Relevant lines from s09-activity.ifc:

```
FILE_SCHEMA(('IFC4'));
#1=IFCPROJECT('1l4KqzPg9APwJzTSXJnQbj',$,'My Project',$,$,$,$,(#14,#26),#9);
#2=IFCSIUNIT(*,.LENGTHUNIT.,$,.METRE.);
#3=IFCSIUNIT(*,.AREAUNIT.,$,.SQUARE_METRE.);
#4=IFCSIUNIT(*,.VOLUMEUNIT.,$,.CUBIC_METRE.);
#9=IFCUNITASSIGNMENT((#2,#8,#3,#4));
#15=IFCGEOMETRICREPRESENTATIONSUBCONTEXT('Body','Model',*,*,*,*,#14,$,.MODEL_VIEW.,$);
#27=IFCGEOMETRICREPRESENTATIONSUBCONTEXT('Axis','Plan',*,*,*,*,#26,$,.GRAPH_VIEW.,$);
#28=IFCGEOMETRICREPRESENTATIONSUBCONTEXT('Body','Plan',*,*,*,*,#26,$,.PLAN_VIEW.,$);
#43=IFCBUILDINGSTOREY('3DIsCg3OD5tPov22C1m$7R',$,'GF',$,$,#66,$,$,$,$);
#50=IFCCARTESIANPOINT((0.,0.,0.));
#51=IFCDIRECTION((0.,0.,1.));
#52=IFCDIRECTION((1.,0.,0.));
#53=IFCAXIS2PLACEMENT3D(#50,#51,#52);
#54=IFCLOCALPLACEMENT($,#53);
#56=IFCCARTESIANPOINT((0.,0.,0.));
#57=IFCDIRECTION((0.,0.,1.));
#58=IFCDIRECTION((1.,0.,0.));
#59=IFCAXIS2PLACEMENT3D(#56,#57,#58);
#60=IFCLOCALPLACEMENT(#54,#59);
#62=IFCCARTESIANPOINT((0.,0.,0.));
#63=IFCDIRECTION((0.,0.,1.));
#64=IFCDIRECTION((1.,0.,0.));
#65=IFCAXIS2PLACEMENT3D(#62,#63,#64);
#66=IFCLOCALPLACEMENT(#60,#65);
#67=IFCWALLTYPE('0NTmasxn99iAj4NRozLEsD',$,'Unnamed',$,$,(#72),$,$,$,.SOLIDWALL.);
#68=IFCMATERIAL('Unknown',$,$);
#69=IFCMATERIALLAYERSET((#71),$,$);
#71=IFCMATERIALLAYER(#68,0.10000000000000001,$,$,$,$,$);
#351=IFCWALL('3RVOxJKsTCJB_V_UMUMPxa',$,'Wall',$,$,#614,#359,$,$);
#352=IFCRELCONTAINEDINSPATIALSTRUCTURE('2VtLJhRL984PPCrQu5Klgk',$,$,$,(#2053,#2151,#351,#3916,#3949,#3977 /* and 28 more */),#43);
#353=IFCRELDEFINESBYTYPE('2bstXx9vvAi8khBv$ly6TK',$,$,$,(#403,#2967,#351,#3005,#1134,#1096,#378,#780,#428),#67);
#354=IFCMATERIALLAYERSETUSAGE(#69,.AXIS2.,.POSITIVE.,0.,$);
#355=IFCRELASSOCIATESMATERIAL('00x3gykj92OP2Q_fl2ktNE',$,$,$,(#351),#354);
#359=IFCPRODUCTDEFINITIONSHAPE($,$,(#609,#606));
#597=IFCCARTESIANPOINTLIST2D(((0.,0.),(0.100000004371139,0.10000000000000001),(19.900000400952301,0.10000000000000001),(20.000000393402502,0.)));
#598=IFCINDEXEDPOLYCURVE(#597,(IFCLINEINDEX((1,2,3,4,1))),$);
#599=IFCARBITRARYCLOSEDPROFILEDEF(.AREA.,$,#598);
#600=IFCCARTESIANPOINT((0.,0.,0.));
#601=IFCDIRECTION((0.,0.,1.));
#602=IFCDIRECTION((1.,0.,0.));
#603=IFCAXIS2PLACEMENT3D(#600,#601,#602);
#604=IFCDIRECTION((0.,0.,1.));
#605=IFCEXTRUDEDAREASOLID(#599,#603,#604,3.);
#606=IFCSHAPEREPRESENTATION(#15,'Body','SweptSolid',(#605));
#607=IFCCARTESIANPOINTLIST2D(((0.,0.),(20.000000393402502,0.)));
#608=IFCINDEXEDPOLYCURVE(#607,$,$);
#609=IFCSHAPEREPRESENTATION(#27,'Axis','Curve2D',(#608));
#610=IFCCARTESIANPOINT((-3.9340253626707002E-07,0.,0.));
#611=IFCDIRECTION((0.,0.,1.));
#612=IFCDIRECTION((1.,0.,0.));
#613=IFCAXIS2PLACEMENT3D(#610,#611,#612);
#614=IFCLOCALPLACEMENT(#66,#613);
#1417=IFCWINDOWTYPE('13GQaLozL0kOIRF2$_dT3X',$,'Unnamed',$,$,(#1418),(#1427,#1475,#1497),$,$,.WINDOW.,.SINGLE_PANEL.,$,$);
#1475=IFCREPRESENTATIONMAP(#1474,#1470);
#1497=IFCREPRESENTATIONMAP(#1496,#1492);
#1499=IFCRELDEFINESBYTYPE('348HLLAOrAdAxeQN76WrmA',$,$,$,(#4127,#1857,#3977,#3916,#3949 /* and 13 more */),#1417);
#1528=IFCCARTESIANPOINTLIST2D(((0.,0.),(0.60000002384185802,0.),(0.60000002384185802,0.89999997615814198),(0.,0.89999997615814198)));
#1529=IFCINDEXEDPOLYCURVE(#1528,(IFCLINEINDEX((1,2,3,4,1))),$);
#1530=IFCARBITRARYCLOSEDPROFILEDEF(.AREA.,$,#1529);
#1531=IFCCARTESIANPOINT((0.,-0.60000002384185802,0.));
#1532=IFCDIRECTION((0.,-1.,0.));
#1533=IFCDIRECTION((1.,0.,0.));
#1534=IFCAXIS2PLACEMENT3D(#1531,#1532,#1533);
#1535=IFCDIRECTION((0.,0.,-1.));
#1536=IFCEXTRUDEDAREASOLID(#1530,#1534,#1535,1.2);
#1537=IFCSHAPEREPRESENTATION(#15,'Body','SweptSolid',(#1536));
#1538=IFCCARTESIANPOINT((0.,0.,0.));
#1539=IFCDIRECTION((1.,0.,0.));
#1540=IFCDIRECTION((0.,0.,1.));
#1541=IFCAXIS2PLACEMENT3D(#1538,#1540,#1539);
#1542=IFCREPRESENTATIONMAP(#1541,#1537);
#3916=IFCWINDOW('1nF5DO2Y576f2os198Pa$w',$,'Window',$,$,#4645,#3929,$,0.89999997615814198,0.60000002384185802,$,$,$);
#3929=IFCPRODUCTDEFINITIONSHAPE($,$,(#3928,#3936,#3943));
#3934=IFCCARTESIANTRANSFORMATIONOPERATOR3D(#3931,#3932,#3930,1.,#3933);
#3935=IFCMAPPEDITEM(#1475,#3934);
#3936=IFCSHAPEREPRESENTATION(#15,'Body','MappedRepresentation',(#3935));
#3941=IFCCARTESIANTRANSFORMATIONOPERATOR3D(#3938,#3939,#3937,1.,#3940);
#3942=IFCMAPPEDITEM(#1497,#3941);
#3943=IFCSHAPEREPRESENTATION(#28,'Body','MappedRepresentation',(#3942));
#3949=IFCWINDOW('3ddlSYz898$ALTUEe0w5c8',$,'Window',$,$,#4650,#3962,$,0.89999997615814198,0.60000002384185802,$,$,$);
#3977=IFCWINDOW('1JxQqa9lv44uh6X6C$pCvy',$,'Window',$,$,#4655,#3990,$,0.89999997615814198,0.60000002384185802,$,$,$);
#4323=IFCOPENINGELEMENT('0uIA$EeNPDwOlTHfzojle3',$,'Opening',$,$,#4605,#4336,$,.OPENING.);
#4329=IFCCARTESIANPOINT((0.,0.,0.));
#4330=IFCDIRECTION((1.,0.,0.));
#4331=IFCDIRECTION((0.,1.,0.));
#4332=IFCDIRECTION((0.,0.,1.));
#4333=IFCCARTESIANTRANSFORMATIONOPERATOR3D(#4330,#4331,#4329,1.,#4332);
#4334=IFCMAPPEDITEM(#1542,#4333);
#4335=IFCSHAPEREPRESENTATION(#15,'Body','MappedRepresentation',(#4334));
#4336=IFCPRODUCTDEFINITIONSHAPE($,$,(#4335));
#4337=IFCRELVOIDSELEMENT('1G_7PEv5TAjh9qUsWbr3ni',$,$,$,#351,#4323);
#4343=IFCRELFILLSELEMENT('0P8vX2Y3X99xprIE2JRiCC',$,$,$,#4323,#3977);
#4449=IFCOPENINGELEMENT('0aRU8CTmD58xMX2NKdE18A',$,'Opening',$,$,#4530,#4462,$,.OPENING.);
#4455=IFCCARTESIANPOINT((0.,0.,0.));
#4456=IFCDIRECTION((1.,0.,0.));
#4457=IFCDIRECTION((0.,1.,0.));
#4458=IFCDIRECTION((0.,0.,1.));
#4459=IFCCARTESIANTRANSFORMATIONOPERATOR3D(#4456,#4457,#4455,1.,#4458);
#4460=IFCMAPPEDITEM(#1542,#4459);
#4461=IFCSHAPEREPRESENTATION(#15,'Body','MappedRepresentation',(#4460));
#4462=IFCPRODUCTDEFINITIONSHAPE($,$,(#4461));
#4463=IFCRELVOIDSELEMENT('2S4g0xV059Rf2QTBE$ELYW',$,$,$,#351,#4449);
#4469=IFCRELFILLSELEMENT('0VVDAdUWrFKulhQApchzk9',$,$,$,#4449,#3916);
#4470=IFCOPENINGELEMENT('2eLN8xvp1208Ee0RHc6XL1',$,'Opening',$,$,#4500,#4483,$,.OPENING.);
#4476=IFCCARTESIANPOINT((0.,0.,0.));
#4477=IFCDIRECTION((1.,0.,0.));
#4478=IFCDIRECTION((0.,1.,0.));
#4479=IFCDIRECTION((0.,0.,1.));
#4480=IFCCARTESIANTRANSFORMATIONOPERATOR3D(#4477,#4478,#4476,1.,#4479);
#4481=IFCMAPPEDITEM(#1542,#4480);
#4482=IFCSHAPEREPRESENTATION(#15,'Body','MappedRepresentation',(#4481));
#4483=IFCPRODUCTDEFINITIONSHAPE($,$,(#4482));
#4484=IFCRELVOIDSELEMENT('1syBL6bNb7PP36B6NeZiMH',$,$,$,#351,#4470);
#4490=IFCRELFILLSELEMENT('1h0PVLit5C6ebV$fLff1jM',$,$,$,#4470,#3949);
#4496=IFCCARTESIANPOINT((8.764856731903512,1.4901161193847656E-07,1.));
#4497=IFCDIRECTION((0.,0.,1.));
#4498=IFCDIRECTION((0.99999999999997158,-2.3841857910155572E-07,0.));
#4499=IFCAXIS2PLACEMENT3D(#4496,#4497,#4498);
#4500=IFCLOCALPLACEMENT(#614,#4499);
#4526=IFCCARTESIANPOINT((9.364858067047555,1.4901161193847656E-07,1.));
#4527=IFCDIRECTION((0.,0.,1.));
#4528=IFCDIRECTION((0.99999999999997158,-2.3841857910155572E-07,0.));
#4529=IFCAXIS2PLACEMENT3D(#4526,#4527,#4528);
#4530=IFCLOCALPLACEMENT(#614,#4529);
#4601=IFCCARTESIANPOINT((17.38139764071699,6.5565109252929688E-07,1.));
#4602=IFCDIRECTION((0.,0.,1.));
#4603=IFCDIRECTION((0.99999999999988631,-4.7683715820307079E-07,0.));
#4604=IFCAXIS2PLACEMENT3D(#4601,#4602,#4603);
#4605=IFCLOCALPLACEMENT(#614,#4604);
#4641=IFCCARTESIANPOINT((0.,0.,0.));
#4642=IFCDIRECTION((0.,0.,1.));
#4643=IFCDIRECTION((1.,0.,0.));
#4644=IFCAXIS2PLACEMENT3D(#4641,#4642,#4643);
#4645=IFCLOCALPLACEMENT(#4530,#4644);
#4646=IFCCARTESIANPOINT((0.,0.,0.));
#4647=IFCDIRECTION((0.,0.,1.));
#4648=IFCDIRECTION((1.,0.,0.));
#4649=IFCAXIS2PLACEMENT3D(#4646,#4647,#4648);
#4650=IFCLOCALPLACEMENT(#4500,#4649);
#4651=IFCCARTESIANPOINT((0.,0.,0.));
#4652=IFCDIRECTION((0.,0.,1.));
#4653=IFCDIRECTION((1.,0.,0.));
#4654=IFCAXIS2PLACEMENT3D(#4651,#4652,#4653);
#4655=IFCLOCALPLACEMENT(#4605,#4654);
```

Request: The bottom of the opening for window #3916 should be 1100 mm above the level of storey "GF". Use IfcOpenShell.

```python
import numpy as np
import ifcopenshell
import ifcopenshell.api.geometry
import ifcopenshell.geom
import ifcopenshell.util.element
import ifcopenshell.util.placement
import ifcopenshell.util.shape
import ifcopenshell.util.unit

model = ifcopenshell.open("s09-activity.ifc")
unit_scale = ifcopenshell.util.unit.calculate_unit_scale(model)

window = model.by_guid("1nF5DO2Y576f2os198Pa$w")
opening = window.FillsVoids[0].RelatingOpeningElement
storey = ifcopenshell.util.element.get_container(window, ifc_class="IfcBuildingStorey")
level = ifcopenshell.util.placement.get_local_placement(storey.ObjectPlacement)[2, 3]

# The opening's origin need not be at the sill, so measure its lowest point.
shape = ifcopenshell.geom.create_shape(ifcopenshell.geom.settings(), opening)
bottom = ifcopenshell.util.shape.get_shape_bottom_elevation(shape, shape.geometry) / unit_scale
dz = level + 1.1 / unit_scale - bottom

shift = np.array([0.0, 0.0, dz])
# The window is placed relative to its opening, so it follows when the opening moves.
matrix = ifcopenshell.util.placement.get_local_placement(opening.ObjectPlacement)
matrix[:3, 3] += shift
ifcopenshell.api.geometry.edit_object_placement(
    model, product=opening, matrix=matrix, is_si=False, should_transform_children=True
)

print(f"moved by {dz * unit_scale:+.3f} m")

model.write("s09-activity_updated.ifc")
```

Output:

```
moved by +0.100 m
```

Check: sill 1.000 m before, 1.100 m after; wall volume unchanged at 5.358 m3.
